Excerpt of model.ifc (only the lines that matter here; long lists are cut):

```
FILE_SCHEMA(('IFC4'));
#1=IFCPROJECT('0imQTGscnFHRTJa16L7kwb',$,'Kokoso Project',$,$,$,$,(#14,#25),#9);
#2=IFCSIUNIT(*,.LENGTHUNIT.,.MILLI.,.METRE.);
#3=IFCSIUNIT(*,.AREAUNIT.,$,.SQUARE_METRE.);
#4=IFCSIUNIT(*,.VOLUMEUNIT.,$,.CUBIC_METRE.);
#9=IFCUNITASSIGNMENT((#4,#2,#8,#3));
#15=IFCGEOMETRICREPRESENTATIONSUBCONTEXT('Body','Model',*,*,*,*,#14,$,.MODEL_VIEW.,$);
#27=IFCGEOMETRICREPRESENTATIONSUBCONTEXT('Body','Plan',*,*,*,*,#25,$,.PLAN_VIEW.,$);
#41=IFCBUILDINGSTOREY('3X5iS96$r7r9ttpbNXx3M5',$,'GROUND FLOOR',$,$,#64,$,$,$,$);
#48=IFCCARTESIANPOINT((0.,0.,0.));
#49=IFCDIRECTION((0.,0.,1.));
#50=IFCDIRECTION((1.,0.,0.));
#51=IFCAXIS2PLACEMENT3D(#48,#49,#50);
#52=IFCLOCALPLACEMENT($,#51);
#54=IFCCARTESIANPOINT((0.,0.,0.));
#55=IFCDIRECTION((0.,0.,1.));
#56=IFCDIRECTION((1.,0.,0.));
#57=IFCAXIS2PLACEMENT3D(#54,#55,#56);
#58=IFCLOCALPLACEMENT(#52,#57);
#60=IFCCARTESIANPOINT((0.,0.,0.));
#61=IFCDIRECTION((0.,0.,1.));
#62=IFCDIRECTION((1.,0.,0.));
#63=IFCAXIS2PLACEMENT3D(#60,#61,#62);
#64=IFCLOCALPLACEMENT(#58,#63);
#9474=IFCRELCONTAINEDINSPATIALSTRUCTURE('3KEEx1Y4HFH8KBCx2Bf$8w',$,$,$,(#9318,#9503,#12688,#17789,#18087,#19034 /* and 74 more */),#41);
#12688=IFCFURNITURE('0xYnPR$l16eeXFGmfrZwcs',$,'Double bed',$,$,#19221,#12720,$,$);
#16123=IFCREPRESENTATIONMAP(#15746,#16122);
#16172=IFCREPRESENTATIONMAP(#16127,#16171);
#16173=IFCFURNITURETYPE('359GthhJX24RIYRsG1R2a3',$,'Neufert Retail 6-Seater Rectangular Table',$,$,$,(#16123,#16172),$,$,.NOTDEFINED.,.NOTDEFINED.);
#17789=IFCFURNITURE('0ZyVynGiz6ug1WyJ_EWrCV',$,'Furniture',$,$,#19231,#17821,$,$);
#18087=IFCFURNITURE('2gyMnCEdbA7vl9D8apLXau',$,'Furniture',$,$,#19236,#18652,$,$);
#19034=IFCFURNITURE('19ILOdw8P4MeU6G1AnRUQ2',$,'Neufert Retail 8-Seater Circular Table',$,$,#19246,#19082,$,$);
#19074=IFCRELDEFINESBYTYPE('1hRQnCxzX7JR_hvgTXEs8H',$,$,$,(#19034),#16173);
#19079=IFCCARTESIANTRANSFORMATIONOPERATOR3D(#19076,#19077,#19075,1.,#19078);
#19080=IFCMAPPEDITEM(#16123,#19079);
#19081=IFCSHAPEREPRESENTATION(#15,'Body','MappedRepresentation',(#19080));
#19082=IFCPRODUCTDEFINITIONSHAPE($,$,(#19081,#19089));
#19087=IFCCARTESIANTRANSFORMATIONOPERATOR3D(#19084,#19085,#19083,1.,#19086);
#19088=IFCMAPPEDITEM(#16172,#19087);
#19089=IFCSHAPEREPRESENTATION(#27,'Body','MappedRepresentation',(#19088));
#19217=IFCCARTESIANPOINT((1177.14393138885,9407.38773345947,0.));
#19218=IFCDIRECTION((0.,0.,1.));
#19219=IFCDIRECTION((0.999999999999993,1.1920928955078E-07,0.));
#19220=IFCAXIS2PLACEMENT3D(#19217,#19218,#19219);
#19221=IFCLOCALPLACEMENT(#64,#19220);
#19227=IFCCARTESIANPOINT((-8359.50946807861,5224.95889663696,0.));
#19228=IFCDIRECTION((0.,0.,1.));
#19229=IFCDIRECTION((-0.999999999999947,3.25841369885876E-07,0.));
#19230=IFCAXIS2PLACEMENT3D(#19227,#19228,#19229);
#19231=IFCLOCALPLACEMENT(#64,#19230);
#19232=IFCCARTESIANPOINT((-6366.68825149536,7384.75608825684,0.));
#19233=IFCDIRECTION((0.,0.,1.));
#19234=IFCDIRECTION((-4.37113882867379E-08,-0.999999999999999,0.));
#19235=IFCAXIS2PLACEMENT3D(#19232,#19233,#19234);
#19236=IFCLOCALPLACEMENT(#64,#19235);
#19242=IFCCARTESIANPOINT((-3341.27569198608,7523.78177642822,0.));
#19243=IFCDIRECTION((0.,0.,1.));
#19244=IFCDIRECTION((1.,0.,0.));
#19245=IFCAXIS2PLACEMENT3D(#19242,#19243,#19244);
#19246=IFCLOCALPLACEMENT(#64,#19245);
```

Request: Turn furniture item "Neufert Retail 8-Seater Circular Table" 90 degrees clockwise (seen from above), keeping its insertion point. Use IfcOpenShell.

```python
import ifcopenshell
import ifcopenshell.api.geometry
import ifcopenshell.util.placement

model = ifcopenshell.open("model.ifc")

item = model.by_guid("19ILOdw8P4MeU6G1AnRUQ2")
matrix = ifcopenshell.util.placement.get_local_placement(item.ObjectPlacement)
matrix = matrix @ ifcopenshell.util.placement.rotation(-90, "Z")
ifcopenshell.api.geometry.edit_object_placement(model, product=item, matrix=matrix, is_si=False)

print(ifcopenshell.util.placement.get_local_placement(item.ObjectPlacement).round(3) + 0.0)

model.write("model_edited.ifc")
```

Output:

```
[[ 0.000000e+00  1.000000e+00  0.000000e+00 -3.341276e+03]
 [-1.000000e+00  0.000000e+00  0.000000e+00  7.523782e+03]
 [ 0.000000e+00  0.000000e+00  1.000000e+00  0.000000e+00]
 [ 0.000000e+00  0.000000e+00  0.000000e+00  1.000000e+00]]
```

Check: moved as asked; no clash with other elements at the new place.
